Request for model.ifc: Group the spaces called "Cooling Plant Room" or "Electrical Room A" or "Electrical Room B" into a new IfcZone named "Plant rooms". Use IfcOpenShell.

First a look at what the model holds.

```python
import ifcopenshell

model = ifcopenshell.open("model.ifc")
print(model.schema)
seen = {}
for space in model.by_type("IfcSpace"):
    seen[space.LongName] = seen.get(space.LongName, 0) + 1
for name, count in sorted(seen.items(), key=str):
    print(count, "x", name)
print("zones:", [z.Name for z in model.by_type("IfcZone")][:20])
```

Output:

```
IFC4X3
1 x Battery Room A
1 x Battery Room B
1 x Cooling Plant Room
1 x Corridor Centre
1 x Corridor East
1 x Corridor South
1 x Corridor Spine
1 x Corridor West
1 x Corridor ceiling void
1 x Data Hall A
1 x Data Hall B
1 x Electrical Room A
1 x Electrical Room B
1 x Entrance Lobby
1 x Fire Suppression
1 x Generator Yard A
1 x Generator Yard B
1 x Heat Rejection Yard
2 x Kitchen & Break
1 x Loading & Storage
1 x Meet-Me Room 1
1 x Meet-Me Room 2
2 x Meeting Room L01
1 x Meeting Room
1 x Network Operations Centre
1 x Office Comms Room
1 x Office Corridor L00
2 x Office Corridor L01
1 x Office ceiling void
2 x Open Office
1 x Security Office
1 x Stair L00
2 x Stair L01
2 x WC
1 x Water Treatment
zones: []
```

```python
import ifcopenshell
import ifcopenshell.api.group
import ifcopenshell.api.root

model = ifcopenshell.open("model.ifc")

names = {"Cooling Plant Room", "Electrical Room A", "Electrical Room B"}
spaces = [s for s in model.by_type("IfcSpace") if s.LongName in names]

zone = ifcopenshell.api.root.create_entity(model, ifc_class="IfcZone", name="Plant rooms")
ifcopenshell.api.group.assign_group(model, products=spaces, group=zone)
print(len(spaces), "spaces in", zone.Name)

model.write("model_rev.ifc")
```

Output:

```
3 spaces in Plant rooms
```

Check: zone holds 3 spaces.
